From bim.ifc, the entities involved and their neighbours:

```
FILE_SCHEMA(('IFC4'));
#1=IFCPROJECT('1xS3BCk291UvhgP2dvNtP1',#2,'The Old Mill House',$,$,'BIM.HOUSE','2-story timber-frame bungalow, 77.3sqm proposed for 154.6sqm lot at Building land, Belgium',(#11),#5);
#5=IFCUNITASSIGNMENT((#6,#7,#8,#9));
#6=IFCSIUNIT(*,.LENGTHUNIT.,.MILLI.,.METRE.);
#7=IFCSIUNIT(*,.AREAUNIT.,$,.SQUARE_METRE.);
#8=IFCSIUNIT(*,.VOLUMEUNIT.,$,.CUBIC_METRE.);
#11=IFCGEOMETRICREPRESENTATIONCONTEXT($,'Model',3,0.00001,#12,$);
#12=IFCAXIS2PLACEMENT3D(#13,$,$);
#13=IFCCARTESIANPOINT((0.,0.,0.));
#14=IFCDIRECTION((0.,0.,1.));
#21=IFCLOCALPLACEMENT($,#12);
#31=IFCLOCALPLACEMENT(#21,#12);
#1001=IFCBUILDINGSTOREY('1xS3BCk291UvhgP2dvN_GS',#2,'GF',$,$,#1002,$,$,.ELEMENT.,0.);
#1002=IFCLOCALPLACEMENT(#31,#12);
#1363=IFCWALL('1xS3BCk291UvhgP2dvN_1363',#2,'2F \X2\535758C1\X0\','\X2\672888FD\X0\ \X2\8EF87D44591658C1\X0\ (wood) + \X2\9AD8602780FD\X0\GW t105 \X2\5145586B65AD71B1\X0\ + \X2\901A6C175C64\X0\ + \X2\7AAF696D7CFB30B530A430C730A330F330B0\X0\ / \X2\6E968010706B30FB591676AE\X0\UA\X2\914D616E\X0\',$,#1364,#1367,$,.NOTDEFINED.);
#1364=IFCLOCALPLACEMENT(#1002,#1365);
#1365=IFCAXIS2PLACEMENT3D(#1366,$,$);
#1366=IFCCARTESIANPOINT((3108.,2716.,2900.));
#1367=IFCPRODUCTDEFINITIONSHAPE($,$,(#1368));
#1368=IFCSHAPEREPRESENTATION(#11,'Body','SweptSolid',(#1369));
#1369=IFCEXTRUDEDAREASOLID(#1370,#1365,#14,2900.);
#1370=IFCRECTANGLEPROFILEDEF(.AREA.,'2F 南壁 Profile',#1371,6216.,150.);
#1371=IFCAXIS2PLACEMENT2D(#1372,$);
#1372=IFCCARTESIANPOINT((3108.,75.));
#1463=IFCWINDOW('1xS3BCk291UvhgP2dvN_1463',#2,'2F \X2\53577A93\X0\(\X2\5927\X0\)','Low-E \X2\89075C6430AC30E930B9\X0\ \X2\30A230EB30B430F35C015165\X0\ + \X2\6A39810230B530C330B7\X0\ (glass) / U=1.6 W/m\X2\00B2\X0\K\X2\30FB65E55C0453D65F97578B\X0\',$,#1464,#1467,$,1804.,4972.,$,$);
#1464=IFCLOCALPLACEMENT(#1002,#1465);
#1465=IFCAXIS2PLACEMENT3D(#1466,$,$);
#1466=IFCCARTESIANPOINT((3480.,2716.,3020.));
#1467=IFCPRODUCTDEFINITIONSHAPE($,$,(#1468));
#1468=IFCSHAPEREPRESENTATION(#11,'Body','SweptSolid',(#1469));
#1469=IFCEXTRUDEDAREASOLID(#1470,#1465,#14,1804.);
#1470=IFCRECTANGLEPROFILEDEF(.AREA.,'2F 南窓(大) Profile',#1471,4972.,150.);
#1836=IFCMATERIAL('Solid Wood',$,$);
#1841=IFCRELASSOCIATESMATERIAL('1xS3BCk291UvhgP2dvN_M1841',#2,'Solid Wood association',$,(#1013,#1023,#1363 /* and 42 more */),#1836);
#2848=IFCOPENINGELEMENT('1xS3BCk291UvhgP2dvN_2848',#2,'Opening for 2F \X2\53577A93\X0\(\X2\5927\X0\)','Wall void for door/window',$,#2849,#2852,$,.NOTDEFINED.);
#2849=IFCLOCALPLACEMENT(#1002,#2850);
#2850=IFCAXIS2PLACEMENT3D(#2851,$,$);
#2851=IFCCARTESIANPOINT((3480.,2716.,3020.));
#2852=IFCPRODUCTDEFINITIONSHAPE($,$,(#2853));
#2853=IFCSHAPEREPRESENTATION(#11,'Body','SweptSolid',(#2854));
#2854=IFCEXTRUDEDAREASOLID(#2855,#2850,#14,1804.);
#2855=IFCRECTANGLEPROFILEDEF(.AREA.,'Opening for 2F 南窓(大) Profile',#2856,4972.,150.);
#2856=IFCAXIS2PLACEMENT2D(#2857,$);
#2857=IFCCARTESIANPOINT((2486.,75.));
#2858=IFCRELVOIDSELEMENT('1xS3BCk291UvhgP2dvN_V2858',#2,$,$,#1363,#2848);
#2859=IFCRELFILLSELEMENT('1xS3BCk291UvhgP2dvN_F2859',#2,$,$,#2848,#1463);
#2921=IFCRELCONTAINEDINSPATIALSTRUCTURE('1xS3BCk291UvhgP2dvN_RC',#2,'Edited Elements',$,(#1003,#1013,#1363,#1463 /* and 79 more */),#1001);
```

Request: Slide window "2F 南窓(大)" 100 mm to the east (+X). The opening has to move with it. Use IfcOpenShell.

```python
import ifcopenshell
import ifcopenshell.api.geometry
import ifcopenshell.util.placement

model = ifcopenshell.open("bim.ifc")

window = model.by_guid("1xS3BCk291UvhgP2dvN_1463")
opening = window.FillsVoids[0].RelatingOpeningElement
wall = opening.VoidsElements[0].RelatingBuildingElement

wall_matrix = ifcopenshell.util.placement.get_local_placement(wall.ObjectPlacement)
shift = wall_matrix[:3, 0] * 100.0
before = ifcopenshell.util.placement.get_local_placement(window.ObjectPlacement)[:3, 3].copy()

# The window is not placed relative to its opening, so move both.
for product in (opening, window):
    matrix = ifcopenshell.util.placement.get_local_placement(product.ObjectPlacement)
    matrix[:3, 3] += shift
    ifcopenshell.api.geometry.edit_object_placement(model, product=product, matrix=matrix, is_si=False)

after = ifcopenshell.util.placement.get_local_placement(window.ObjectPlacement)[:3, 3]
print("window moved by", (after - before).round(3) + 0.0)

model.write("bim_updated.ifc")
```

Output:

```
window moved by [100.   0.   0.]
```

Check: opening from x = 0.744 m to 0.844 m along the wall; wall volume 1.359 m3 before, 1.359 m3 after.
